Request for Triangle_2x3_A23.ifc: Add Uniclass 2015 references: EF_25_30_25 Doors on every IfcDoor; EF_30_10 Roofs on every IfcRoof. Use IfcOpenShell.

First a look at what the model holds.

```python
import ifcopenshell

model = ifcopenshell.open("Triangle_2x3_A23.ifc")
print(model.schema)
print("classifications:", [c.Name for c in model.by_type("IfcClassification")])
for ifc_class in ("IfcDoor", "IfcRoof", "IfcStair", "IfcWall", "IfcWindow"):
    print(ifc_class, len(model.by_type(ifc_class)))
```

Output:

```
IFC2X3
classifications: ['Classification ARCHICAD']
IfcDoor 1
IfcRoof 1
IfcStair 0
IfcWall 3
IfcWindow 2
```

```python
import ifcopenshell
import ifcopenshell.api.classification

model = ifcopenshell.open("Triangle_2x3_A23.ifc")

# IFC2X3 requires Source and Edition and has no link from the project to the system.
system = model.create_entity("IfcClassification", Source="NBS", Edition="2015", Name="Uniclass 2015")

codes = {
    "IfcDoor": ("EF_25_30_25", "Doors"),
    "IfcRoof": ("EF_30_10", "Roofs"),
}
for ifc_class, (code, name) in codes.items():
    products = model.by_type(ifc_class)
    ifcopenshell.api.classification.add_reference(
        model, products=products, classification=system, identification=code, name=name
    )
    print(code, len(products))

model.write("Triangle_2x3_A23_v2.ifc")
```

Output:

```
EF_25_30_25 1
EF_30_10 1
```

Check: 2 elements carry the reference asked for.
